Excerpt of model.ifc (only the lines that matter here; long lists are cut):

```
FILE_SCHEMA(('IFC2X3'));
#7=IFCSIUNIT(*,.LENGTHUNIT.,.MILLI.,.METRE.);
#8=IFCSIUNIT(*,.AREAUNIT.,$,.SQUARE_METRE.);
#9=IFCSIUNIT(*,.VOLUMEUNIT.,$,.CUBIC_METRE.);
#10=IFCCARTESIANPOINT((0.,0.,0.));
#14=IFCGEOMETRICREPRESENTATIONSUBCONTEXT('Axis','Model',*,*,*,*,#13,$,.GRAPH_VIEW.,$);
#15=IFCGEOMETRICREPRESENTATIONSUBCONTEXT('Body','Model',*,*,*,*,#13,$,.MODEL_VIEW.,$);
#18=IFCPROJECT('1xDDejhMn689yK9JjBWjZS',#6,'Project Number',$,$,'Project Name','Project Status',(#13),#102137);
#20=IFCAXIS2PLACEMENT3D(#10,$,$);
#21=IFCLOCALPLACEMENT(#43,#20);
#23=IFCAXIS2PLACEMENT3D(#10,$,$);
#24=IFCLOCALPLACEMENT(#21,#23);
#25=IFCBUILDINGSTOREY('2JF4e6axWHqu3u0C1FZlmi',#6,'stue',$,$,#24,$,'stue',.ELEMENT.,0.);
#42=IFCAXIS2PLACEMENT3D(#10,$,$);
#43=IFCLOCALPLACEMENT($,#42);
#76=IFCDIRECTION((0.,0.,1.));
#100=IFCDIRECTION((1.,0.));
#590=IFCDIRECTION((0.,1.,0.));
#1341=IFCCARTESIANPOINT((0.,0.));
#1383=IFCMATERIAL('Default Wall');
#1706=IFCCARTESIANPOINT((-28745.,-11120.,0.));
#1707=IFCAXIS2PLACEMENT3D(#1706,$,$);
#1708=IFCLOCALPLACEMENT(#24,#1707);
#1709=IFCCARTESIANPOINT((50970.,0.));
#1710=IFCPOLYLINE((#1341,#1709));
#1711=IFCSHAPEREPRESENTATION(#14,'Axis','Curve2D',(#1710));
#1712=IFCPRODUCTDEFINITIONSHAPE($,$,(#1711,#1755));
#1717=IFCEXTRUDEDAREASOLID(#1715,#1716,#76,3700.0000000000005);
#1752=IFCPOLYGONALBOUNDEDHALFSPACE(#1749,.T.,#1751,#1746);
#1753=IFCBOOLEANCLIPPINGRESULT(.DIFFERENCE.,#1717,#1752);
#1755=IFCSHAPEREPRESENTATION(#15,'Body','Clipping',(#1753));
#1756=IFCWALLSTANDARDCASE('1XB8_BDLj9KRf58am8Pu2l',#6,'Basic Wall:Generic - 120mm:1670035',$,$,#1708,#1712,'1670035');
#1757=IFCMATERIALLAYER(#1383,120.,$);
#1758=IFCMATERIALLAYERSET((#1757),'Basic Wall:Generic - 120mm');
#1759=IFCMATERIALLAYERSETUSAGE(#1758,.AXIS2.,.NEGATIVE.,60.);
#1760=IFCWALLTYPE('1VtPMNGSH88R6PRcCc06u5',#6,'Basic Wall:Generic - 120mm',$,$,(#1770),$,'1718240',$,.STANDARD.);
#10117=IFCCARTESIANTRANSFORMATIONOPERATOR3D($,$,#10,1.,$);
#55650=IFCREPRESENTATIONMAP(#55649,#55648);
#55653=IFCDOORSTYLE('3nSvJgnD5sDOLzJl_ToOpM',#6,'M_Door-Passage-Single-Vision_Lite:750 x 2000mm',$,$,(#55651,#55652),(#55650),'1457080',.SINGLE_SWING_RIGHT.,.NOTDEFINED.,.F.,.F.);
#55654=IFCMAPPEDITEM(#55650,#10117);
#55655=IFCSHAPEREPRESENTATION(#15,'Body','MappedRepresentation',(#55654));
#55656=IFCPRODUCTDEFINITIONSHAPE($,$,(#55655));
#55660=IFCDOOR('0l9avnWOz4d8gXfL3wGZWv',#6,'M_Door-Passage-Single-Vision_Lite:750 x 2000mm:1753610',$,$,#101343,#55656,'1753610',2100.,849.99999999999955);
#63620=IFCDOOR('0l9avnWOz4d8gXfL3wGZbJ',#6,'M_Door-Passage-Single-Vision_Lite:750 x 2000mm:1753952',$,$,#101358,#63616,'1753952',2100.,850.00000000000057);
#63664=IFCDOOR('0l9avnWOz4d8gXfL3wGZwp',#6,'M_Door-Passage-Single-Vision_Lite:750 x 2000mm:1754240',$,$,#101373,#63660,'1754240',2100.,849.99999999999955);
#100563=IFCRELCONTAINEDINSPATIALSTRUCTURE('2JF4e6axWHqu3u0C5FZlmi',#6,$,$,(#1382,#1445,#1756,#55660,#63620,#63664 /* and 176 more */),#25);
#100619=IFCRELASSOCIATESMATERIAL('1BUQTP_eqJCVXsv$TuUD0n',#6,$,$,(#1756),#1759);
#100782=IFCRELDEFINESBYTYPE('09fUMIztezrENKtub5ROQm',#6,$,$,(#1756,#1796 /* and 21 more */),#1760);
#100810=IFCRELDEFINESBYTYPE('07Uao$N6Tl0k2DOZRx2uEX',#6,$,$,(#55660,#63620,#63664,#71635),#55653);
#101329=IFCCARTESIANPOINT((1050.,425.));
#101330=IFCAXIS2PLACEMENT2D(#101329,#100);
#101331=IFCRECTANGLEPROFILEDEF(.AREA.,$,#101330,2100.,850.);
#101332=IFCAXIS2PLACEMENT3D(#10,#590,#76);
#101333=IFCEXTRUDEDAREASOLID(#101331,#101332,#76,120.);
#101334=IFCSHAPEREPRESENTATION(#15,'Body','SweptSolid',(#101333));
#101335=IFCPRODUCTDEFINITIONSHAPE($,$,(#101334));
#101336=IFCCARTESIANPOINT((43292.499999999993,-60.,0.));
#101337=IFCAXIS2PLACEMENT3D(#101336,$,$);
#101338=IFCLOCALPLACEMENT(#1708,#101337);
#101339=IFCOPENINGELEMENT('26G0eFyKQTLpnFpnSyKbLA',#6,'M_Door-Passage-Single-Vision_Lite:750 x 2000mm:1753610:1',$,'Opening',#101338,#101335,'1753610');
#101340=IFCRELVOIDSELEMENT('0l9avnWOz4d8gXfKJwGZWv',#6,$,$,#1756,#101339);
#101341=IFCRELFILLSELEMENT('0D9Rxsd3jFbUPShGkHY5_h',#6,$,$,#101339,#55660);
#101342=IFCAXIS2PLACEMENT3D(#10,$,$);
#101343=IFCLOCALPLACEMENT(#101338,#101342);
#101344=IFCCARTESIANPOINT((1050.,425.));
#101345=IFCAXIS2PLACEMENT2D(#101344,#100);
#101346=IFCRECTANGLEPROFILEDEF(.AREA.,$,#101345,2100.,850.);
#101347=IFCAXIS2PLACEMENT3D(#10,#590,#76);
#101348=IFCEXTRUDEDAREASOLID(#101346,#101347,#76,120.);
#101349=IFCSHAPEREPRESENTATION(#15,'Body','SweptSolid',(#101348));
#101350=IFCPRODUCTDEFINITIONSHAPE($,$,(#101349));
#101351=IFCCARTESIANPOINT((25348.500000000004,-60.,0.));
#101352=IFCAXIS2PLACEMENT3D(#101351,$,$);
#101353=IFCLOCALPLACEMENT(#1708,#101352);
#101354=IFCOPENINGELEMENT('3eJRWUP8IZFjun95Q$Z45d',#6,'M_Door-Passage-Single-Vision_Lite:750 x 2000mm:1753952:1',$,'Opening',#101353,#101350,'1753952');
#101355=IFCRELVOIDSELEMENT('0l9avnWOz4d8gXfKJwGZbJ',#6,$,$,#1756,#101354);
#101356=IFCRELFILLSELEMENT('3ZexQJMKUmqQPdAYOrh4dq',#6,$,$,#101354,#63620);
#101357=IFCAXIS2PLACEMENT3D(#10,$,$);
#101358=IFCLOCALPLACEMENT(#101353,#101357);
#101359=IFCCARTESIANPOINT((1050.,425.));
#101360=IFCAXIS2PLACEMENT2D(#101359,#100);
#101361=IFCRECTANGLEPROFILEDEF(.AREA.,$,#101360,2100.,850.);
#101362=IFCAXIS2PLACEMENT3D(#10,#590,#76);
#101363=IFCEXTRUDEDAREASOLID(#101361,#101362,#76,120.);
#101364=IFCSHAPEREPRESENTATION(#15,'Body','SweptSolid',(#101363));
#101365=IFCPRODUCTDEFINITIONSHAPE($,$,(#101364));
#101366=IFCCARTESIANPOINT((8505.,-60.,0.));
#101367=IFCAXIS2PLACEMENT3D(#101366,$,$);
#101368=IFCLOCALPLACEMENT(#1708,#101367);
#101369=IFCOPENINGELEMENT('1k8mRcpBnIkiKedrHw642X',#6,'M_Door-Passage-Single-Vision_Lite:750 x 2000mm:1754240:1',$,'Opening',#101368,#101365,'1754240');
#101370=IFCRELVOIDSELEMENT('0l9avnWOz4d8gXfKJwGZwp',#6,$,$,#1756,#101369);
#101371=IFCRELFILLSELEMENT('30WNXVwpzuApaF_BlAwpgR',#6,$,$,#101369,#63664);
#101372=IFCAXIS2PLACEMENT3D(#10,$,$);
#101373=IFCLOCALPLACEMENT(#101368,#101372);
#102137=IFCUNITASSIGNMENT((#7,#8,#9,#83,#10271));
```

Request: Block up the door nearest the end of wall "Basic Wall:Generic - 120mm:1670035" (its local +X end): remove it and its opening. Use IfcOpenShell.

```python
import ifcopenshell
import ifcopenshell.api.feature
import ifcopenshell.api.root
import ifcopenshell.geom
import ifcopenshell.util.shape

model = ifcopenshell.open("model.ifc")
settings = ifcopenshell.geom.settings()


def volume(element):
    """Net volume in cubic metres, openings subtracted."""
    shape = ifcopenshell.geom.create_shape(settings, element)
    return ifcopenshell.util.shape.get_volume(shape.geometry)


door = model.by_id(55660)
opening = door.FillsVoids[0].RelatingOpeningElement
wall = opening.VoidsElements[0].RelatingBuildingElement
before = volume(wall)

ifcopenshell.api.root.remove_product(model, product=door)
ifcopenshell.api.feature.remove_feature(model, feature=opening)

after = volume(wall)

print(f"wall volume {before:.3f} -> {after:.3f} m3")

model.write("model_updated.ifc")
```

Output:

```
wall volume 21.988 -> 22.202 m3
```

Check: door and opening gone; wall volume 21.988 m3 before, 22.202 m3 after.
